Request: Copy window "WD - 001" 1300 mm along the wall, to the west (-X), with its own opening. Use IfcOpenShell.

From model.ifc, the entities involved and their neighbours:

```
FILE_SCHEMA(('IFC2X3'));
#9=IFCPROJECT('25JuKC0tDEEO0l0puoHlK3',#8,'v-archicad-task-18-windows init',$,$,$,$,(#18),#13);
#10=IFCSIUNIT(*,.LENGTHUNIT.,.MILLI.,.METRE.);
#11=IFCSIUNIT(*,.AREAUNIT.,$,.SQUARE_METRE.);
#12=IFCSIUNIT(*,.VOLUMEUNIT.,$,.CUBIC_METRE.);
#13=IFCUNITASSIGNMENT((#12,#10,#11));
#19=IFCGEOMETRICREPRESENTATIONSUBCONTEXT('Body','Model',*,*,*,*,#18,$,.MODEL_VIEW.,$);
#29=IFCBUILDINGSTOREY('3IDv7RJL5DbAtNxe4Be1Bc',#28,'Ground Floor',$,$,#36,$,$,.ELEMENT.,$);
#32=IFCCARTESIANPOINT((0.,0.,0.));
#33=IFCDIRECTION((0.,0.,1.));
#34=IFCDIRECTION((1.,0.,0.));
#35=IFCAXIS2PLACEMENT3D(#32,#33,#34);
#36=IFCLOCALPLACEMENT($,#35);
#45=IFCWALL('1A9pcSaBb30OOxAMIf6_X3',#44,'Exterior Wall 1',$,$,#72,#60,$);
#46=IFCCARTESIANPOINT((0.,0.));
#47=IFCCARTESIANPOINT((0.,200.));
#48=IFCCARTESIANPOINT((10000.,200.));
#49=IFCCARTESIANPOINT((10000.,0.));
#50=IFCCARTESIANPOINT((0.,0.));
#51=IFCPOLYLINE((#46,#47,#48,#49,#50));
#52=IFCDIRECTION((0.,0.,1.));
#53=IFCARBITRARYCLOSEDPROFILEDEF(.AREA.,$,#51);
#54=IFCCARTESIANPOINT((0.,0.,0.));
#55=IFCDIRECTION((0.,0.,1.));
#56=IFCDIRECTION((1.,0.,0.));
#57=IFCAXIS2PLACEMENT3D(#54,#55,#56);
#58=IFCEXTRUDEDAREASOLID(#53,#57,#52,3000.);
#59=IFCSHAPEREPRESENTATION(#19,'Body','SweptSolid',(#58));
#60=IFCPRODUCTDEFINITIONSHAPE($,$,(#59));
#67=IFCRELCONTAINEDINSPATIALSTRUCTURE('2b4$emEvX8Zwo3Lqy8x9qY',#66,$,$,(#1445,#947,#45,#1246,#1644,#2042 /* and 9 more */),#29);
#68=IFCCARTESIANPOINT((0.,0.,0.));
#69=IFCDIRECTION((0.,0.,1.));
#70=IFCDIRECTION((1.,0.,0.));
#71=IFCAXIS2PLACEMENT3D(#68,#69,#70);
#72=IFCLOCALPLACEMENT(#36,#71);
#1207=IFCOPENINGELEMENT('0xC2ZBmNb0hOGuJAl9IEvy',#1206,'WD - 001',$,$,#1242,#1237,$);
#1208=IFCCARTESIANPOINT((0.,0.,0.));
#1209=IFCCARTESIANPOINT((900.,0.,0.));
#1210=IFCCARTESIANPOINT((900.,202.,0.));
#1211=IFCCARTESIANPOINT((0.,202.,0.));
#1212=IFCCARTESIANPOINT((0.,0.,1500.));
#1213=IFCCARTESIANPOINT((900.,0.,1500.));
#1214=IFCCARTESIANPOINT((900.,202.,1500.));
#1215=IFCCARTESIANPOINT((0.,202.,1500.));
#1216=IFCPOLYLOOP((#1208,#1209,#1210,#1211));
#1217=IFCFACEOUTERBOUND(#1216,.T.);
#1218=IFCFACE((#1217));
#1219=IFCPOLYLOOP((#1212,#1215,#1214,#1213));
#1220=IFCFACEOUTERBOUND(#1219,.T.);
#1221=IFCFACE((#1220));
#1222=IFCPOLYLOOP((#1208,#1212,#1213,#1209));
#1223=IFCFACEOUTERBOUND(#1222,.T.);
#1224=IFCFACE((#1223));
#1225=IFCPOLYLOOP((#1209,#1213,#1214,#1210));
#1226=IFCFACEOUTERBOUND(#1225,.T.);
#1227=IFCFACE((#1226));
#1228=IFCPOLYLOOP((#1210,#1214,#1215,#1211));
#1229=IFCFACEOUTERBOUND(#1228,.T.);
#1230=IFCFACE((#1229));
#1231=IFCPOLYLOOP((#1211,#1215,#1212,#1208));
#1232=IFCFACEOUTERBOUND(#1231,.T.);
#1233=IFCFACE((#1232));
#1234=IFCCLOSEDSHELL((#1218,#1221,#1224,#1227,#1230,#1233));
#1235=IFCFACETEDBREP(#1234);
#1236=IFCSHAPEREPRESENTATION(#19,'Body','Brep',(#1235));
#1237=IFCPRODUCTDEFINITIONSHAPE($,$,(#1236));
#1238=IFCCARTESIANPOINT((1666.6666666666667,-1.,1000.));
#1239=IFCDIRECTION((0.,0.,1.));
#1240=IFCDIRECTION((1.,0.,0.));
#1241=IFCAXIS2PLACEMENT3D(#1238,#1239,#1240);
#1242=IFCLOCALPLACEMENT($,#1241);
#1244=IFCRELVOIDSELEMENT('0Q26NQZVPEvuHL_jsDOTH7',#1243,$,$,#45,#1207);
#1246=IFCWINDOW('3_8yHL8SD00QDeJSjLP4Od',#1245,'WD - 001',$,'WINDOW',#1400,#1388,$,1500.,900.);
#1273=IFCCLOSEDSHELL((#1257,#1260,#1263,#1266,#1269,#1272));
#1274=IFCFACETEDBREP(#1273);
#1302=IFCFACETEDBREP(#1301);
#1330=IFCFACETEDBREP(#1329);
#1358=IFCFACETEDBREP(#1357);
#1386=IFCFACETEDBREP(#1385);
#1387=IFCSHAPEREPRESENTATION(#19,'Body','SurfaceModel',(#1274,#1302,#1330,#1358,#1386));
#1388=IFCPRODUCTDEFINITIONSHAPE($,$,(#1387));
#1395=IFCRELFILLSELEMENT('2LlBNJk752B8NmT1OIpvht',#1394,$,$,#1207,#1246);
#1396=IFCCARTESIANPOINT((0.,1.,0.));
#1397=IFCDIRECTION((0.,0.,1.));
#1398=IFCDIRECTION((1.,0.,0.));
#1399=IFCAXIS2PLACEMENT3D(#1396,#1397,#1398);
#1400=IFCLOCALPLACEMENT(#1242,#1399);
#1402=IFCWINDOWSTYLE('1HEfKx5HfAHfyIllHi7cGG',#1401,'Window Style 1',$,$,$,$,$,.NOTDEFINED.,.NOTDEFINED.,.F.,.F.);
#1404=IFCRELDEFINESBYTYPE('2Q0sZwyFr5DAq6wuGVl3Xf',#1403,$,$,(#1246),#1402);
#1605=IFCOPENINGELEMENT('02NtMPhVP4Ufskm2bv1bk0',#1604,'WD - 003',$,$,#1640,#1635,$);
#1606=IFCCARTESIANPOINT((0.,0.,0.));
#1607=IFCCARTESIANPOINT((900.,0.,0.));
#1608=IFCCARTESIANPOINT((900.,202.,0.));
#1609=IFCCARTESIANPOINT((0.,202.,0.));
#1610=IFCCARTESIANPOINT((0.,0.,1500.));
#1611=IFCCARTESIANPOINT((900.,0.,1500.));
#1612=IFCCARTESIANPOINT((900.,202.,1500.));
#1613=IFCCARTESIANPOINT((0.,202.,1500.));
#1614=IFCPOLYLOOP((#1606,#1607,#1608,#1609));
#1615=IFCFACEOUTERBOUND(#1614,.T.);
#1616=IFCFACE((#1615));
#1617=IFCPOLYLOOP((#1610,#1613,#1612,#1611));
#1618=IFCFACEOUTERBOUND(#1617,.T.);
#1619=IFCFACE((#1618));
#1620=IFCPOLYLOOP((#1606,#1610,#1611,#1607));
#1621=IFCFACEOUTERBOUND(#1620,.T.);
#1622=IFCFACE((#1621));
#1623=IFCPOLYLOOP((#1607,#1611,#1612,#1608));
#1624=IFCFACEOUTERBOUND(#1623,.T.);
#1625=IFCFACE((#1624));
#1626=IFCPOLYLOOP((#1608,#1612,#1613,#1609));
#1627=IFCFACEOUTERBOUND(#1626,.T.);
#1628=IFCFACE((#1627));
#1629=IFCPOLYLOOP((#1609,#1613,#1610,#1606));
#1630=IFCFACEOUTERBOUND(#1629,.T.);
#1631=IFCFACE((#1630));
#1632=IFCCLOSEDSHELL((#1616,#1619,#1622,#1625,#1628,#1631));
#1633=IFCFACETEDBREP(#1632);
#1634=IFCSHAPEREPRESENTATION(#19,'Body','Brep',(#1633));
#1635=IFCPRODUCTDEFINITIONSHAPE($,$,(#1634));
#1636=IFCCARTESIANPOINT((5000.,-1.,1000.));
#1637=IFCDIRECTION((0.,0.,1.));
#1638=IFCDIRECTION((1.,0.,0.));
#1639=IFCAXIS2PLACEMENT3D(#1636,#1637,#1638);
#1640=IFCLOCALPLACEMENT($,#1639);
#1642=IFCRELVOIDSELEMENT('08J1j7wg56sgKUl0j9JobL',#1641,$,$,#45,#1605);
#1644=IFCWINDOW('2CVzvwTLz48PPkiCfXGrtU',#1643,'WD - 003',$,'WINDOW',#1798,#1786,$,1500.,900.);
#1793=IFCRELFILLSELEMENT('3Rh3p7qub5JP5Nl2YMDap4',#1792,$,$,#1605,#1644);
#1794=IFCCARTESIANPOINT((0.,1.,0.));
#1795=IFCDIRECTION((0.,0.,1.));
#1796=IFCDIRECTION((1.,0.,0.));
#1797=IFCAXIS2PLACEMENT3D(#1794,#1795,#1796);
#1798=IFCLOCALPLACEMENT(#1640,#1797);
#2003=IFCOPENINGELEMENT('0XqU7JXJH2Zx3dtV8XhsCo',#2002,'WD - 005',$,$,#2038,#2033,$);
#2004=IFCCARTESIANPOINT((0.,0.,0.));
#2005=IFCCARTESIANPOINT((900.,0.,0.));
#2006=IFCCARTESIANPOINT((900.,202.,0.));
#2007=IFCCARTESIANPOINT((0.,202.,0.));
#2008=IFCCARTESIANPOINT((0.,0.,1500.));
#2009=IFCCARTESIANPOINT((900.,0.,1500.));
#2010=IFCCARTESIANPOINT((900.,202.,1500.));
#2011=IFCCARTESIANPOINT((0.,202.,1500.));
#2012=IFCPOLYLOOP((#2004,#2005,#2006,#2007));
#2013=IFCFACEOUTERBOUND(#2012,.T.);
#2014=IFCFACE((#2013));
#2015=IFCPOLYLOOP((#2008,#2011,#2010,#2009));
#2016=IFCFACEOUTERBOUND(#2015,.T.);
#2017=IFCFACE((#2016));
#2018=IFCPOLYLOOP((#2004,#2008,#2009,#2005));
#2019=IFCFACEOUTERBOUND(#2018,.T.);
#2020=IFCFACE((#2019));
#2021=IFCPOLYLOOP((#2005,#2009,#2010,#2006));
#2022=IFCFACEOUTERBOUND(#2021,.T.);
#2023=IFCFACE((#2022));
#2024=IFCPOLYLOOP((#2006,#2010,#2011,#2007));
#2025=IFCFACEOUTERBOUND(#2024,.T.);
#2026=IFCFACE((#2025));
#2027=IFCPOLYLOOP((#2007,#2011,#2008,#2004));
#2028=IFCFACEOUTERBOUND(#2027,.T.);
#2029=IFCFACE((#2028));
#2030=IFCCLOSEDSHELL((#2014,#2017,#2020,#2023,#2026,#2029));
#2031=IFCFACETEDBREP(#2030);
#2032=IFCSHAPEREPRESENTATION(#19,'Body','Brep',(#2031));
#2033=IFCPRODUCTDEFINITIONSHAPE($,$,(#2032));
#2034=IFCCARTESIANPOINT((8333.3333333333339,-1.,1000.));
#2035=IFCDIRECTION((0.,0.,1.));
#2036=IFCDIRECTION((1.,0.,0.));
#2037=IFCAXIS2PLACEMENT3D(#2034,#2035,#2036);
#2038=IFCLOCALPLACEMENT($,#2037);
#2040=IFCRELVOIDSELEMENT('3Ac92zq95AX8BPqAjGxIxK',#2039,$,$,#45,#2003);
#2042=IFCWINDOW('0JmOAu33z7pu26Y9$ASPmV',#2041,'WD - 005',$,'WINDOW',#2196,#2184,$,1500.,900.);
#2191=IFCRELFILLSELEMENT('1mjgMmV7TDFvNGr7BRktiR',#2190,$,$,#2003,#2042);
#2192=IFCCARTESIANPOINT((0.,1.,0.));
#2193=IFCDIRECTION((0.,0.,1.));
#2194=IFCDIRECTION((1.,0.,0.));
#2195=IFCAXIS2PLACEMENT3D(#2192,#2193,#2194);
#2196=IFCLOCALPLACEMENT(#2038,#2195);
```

```python
import ifcopenshell
import ifcopenshell.api.feature
import ifcopenshell.api.geometry
import ifcopenshell.api.root
import ifcopenshell.geom
import ifcopenshell.util.element
import ifcopenshell.util.placement
import ifcopenshell.util.shape

model = ifcopenshell.open("model.ifc")
settings = ifcopenshell.geom.settings()


def volume(element):
    """Net volume in cubic metres, openings subtracted."""
    shape = ifcopenshell.geom.create_shape(settings, element)
    return ifcopenshell.util.shape.get_volume(shape.geometry)


window = model.by_guid("3_8yHL8SD00QDeJSjLP4Od")
opening = window.FillsVoids[0].RelatingOpeningElement
wall = opening.VoidsElements[0].RelatingBuildingElement
before = volume(wall)
shift = ifcopenshell.util.placement.get_local_placement(wall.ObjectPlacement)[:3, 0] * -1300.0

# copy_class copies the void relationship, type, container and properties, but no geometry.
new_opening = ifcopenshell.api.root.copy_class(model, product=opening)
new_opening.Representation = ifcopenshell.util.element.copy_deep(
    model, opening.Representation, exclude=["IfcGeometricRepresentationContext", "IfcRepresentationMap"]
)
new_window = ifcopenshell.api.root.copy_class(model, product=window)
new_window.Representation = ifcopenshell.util.element.copy_deep(
    model, window.Representation, exclude=["IfcGeometricRepresentationContext", "IfcRepresentationMap"]
)
fills = ifcopenshell.api.feature.add_filling(model, opening=new_opening, element=new_window)
fills.OwnerHistory = new_window.OwnerHistory  # required in IFC2X3

for old, new in ((opening, new_opening), (window, new_window)):
    matrix = ifcopenshell.util.placement.get_local_placement(old.ObjectPlacement)
    matrix[:3, 3] += shift
    ifcopenshell.api.geometry.edit_object_placement(model, product=new, matrix=matrix, is_si=False)

after = volume(wall)

print(f"wall volume {before:.3f} -> {after:.3f} m3")

model.write("model_edited.ifc")
```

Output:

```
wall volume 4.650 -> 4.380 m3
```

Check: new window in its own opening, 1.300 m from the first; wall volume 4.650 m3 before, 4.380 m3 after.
